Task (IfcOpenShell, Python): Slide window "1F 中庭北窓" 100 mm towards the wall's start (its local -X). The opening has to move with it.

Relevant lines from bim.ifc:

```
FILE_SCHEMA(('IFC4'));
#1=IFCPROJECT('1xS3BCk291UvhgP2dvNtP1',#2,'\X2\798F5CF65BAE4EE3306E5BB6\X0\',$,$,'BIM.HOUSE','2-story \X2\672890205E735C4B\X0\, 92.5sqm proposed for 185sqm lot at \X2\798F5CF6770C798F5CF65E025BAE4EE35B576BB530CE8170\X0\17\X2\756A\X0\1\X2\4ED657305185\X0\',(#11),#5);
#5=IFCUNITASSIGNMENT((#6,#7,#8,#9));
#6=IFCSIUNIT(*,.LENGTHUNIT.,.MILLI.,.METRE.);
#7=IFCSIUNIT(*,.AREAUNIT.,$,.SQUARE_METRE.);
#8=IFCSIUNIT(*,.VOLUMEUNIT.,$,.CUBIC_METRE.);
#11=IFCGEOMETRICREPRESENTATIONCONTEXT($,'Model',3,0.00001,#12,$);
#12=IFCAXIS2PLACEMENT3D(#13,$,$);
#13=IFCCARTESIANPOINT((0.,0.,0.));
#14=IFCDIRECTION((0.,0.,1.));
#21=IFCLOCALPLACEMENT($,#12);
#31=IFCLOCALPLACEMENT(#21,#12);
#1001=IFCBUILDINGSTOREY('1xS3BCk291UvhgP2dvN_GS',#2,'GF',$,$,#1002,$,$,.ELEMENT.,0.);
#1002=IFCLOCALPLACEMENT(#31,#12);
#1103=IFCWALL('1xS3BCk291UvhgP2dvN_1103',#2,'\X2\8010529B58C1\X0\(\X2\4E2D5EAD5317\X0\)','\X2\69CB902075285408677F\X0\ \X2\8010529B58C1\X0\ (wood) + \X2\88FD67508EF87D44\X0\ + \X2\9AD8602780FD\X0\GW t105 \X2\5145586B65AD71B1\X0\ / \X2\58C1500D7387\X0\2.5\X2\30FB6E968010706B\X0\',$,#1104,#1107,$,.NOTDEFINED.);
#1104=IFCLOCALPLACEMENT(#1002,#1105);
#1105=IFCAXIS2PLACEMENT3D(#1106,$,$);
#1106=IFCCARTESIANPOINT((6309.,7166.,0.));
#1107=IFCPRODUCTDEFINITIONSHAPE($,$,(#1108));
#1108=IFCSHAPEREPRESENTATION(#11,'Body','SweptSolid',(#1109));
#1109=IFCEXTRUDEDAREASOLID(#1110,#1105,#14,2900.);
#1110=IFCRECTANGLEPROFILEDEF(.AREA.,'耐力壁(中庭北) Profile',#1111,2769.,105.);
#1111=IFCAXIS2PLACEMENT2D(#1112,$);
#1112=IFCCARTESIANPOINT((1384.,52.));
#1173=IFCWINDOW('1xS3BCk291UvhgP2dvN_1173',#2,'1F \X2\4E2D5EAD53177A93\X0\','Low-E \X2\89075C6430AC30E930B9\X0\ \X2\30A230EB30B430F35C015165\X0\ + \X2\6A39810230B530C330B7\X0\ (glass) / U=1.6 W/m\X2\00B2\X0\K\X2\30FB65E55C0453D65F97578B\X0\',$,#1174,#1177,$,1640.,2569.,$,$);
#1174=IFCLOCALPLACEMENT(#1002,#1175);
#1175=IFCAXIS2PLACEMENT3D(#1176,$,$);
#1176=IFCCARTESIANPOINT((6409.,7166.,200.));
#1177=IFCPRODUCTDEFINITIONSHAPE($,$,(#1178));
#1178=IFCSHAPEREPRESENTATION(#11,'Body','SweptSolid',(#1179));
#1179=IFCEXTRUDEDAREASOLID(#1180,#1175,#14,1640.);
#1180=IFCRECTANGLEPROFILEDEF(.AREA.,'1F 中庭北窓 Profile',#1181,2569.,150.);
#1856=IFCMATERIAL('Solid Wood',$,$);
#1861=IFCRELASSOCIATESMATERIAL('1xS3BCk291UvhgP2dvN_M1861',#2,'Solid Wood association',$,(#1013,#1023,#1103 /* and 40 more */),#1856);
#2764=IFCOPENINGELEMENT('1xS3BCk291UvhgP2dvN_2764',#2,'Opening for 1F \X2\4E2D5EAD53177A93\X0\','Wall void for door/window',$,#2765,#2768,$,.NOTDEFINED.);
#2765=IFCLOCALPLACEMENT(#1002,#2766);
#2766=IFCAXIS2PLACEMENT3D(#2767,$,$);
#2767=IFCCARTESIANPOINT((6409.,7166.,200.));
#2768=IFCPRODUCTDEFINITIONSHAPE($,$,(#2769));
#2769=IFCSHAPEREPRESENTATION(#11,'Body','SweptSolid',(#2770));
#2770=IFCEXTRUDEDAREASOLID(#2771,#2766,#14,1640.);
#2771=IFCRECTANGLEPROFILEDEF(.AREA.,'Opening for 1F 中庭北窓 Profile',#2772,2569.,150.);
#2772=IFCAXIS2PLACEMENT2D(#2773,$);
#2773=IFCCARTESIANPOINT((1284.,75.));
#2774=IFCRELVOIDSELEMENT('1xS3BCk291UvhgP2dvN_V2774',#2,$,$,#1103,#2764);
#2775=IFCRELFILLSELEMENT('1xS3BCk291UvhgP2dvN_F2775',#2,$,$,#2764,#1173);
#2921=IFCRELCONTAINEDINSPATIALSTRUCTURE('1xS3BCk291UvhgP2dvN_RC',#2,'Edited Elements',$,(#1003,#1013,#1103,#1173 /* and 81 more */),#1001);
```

```python
import ifcopenshell
import ifcopenshell.api.geometry
import ifcopenshell.util.placement

model = ifcopenshell.open("bim.ifc")

window = model.by_guid("1xS3BCk291UvhgP2dvN_1173")
opening = window.FillsVoids[0].RelatingOpeningElement
wall = opening.VoidsElements[0].RelatingBuildingElement

wall_matrix = ifcopenshell.util.placement.get_local_placement(wall.ObjectPlacement)
shift = wall_matrix[:3, 0] * -100.0
before = ifcopenshell.util.placement.get_local_placement(window.ObjectPlacement)[:3, 3].copy()

# The window is not placed relative to its opening, so move both.
for product in (opening, window):
    matrix = ifcopenshell.util.placement.get_local_placement(product.ObjectPlacement)
    matrix[:3, 3] += shift
    ifcopenshell.api.geometry.edit_object_placement(model, product=product, matrix=matrix, is_si=False)

after = ifcopenshell.util.placement.get_local_placement(window.ObjectPlacement)[:3, 3]
print("window moved by", (after - before).round(3) + 0.0)

model.write("bim_edited.ifc")
```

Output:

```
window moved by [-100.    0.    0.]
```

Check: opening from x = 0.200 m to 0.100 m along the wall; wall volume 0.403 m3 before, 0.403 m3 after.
